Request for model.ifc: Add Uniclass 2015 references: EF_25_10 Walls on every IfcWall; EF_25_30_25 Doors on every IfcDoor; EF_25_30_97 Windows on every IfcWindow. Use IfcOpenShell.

First a look at what the model holds.

```python
import ifcopenshell

model = ifcopenshell.open("model.ifc")
print(model.schema)
print("classifications:", [c.Name for c in model.by_type("IfcClassification")])
for ifc_class in ("IfcDoor", "IfcRoof", "IfcStair", "IfcWall", "IfcWindow"):
    print(ifc_class, len(model.by_type(ifc_class)))
```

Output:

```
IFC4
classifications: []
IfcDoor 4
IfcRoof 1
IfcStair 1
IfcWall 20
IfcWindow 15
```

```python
import ifcopenshell
import ifcopenshell.api.classification

model = ifcopenshell.open("model.ifc")

system = ifcopenshell.api.classification.add_classification(model, classification="Uniclass 2015")

codes = {
    "IfcWall": ("EF_25_10", "Walls"),
    "IfcDoor": ("EF_25_30_25", "Doors"),
    "IfcWindow": ("EF_25_30_97", "Windows"),
}
for ifc_class, (code, name) in codes.items():
    products = model.by_type(ifc_class)
    ifcopenshell.api.classification.add_reference(
        model, products=products, classification=system, identification=code, name=name
    )
    print(code, len(products))

model.write("model_edited.ifc")
```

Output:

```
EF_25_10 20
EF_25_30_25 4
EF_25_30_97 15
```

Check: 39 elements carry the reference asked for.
